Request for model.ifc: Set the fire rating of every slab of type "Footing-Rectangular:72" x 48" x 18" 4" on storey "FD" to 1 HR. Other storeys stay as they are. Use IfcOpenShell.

First a look at what the model holds.

```python
import ifcopenshell
import ifcopenshell.util.element

model = ifcopenshell.open("model.ifc")
print(model.schema)
storey = next(s for s in model.by_type("IfcBuildingStorey") if s.Name == "FD")
slabs = [e for e in ifcopenshell.util.element.get_decomposition(storey) if e.is_a("IfcSlab")]
seen = {}
for e in slabs:
    element_type = ifcopenshell.util.element.get_type(e)
    key = (element_type.Name if element_type != e and element_type else None, ifcopenshell.util.element.get_pset(e, "Pset_SlabCommon", "FireRating"))
    seen[key] = seen.get(key, 0) + 1
for (name, value), count in sorted(seen.items(), key=str):
    print(count, "x", name, "|", value)
```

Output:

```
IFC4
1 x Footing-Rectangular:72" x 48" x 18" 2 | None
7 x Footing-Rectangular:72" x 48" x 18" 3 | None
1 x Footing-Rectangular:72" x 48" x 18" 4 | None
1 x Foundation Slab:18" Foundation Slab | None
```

```python
import ifcopenshell
import ifcopenshell.api.pset
import ifcopenshell.util.element

model = ifcopenshell.open("model.ifc")

storey = next(s for s in model.by_type("IfcBuildingStorey") if s.Name == "FD")
slabs = [e for e in ifcopenshell.util.element.get_decomposition(storey) if e.is_a("IfcSlab")]

count = 0
for e in slabs:
    element_type = ifcopenshell.util.element.get_type(e)
    if element_type in (None, e) or element_type.Name != 'Footing-Rectangular:72" x 48" x 18" 4':
        continue
    # add_pset returns the element's existing set when there is one.
    pset = ifcopenshell.api.pset.add_pset(model, product=e, name="Pset_SlabCommon")
    ifcopenshell.api.pset.edit_pset(model, pset=pset, properties={"FireRating": "1 HR"})
    count += 1

print(count, "slabs updated")

model.write("model_v2.ifc")
```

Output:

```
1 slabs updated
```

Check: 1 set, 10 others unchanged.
